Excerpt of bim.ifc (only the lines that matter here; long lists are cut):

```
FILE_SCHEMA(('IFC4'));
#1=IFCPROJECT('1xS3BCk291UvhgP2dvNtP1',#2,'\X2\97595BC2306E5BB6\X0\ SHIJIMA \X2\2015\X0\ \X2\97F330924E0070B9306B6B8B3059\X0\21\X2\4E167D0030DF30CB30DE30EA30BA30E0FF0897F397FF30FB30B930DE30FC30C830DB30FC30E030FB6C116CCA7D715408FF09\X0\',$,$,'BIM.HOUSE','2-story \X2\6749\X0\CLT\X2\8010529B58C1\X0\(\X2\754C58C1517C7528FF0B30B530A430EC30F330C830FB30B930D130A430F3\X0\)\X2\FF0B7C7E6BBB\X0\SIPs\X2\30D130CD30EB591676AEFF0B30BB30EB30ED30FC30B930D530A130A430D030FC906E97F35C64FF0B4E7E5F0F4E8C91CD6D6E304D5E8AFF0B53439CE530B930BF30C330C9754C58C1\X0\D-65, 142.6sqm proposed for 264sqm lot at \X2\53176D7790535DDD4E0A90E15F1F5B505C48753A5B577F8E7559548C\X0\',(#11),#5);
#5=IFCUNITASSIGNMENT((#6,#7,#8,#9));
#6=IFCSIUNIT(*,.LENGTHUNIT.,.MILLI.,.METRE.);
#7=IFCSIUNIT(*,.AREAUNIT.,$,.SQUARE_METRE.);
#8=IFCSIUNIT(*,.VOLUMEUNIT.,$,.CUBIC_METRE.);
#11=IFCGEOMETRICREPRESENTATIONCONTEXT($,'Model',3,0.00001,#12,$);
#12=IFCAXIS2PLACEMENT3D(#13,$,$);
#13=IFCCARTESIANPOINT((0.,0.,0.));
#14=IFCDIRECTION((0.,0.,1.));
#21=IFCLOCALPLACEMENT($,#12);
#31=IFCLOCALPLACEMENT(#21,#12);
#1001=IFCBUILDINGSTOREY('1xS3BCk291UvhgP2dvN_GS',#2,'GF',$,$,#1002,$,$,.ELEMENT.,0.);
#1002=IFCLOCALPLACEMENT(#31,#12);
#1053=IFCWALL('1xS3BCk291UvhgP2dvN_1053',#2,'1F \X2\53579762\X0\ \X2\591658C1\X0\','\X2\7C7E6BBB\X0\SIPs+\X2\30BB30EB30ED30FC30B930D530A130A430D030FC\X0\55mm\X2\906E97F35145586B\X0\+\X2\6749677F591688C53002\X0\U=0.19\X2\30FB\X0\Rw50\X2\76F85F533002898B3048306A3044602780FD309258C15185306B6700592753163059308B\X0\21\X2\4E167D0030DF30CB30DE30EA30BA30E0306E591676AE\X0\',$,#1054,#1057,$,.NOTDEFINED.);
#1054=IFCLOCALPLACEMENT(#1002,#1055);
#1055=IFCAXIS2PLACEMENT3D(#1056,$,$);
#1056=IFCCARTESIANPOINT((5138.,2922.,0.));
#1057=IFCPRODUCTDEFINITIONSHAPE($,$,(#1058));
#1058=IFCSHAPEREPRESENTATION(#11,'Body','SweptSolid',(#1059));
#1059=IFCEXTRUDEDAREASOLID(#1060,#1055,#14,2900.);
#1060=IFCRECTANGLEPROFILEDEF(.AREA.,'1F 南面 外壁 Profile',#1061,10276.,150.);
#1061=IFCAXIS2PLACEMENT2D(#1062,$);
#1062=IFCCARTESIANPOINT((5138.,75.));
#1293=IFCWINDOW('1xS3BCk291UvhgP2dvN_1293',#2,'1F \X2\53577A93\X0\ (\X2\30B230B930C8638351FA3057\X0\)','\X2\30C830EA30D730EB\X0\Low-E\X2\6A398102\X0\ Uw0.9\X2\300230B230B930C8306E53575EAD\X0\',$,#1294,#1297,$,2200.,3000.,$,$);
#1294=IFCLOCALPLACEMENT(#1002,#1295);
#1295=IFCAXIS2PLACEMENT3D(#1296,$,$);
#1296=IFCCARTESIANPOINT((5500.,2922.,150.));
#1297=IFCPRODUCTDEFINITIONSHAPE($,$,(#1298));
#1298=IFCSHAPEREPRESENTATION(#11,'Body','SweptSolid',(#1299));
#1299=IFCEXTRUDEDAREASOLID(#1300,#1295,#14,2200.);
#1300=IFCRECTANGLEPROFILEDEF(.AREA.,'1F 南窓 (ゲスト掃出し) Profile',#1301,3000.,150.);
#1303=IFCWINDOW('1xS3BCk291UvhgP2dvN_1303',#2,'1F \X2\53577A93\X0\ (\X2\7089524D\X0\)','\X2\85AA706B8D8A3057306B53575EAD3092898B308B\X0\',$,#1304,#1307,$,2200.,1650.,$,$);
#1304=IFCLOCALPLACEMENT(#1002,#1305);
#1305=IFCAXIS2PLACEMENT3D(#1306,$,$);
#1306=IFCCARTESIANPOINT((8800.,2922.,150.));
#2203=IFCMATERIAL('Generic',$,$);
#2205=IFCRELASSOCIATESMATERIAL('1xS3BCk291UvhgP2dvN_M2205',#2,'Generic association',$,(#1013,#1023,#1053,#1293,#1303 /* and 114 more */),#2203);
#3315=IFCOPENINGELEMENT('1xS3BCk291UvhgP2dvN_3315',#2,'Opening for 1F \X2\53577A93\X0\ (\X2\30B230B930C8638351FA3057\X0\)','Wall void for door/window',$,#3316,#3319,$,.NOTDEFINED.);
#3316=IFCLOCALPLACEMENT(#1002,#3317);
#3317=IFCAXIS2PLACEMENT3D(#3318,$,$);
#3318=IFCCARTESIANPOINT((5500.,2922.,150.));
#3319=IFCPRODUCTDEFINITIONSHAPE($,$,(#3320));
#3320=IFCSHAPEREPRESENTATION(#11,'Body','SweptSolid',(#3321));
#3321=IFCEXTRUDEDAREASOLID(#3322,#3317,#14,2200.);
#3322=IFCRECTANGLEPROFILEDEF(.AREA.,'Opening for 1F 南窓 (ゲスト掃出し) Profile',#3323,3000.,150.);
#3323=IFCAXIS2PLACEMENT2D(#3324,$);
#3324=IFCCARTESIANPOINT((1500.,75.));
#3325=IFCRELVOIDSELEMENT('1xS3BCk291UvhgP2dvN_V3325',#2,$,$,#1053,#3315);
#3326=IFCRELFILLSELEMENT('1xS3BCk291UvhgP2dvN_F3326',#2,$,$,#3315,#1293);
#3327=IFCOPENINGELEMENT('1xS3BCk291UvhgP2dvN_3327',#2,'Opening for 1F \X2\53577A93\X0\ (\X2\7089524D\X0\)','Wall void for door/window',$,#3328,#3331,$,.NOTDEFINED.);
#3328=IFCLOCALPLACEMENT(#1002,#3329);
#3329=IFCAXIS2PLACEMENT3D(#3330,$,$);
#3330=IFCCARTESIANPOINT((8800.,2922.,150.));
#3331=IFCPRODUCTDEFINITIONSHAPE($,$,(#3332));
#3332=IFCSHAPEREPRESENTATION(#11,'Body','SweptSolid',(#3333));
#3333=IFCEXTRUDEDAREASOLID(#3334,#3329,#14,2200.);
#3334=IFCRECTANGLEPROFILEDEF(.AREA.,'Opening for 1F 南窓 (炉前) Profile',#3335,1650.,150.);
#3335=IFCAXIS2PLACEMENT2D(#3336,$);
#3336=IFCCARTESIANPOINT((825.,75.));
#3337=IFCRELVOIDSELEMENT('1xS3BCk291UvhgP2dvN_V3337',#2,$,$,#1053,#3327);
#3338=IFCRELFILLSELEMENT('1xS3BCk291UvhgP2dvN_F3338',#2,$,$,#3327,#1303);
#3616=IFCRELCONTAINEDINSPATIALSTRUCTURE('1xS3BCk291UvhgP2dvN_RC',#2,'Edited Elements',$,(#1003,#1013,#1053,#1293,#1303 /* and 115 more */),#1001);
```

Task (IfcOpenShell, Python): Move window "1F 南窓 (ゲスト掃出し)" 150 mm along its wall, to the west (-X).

```python
import ifcopenshell
import ifcopenshell.api.geometry
import ifcopenshell.util.placement
import ifcopenshell.util.unit

model = ifcopenshell.open("bim.ifc")
unit_scale = ifcopenshell.util.unit.calculate_unit_scale(model)

window = model.by_id(1293)
opening = window.FillsVoids[0].RelatingOpeningElement
wall = opening.VoidsElements[0].RelatingBuildingElement

wall_matrix = ifcopenshell.util.placement.get_local_placement(wall.ObjectPlacement)
shift = wall_matrix[:3, 0] * -0.15 / unit_scale
before = ifcopenshell.util.placement.get_local_placement(window.ObjectPlacement)[:3, 3].copy()

# The window is not placed relative to its opening, so move both.
for product in (opening, window):
    matrix = ifcopenshell.util.placement.get_local_placement(product.ObjectPlacement)
    matrix[:3, 3] += shift
    ifcopenshell.api.geometry.edit_object_placement(model, product=product, matrix=matrix, is_si=False)

after = ifcopenshell.util.placement.get_local_placement(window.ObjectPlacement)[:3, 3]
print("window moved by", (after - before).round(3) + 0.0)

model.write("bim_rev.ifc")
```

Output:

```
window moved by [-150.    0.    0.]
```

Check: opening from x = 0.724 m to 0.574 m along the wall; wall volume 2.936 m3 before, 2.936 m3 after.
